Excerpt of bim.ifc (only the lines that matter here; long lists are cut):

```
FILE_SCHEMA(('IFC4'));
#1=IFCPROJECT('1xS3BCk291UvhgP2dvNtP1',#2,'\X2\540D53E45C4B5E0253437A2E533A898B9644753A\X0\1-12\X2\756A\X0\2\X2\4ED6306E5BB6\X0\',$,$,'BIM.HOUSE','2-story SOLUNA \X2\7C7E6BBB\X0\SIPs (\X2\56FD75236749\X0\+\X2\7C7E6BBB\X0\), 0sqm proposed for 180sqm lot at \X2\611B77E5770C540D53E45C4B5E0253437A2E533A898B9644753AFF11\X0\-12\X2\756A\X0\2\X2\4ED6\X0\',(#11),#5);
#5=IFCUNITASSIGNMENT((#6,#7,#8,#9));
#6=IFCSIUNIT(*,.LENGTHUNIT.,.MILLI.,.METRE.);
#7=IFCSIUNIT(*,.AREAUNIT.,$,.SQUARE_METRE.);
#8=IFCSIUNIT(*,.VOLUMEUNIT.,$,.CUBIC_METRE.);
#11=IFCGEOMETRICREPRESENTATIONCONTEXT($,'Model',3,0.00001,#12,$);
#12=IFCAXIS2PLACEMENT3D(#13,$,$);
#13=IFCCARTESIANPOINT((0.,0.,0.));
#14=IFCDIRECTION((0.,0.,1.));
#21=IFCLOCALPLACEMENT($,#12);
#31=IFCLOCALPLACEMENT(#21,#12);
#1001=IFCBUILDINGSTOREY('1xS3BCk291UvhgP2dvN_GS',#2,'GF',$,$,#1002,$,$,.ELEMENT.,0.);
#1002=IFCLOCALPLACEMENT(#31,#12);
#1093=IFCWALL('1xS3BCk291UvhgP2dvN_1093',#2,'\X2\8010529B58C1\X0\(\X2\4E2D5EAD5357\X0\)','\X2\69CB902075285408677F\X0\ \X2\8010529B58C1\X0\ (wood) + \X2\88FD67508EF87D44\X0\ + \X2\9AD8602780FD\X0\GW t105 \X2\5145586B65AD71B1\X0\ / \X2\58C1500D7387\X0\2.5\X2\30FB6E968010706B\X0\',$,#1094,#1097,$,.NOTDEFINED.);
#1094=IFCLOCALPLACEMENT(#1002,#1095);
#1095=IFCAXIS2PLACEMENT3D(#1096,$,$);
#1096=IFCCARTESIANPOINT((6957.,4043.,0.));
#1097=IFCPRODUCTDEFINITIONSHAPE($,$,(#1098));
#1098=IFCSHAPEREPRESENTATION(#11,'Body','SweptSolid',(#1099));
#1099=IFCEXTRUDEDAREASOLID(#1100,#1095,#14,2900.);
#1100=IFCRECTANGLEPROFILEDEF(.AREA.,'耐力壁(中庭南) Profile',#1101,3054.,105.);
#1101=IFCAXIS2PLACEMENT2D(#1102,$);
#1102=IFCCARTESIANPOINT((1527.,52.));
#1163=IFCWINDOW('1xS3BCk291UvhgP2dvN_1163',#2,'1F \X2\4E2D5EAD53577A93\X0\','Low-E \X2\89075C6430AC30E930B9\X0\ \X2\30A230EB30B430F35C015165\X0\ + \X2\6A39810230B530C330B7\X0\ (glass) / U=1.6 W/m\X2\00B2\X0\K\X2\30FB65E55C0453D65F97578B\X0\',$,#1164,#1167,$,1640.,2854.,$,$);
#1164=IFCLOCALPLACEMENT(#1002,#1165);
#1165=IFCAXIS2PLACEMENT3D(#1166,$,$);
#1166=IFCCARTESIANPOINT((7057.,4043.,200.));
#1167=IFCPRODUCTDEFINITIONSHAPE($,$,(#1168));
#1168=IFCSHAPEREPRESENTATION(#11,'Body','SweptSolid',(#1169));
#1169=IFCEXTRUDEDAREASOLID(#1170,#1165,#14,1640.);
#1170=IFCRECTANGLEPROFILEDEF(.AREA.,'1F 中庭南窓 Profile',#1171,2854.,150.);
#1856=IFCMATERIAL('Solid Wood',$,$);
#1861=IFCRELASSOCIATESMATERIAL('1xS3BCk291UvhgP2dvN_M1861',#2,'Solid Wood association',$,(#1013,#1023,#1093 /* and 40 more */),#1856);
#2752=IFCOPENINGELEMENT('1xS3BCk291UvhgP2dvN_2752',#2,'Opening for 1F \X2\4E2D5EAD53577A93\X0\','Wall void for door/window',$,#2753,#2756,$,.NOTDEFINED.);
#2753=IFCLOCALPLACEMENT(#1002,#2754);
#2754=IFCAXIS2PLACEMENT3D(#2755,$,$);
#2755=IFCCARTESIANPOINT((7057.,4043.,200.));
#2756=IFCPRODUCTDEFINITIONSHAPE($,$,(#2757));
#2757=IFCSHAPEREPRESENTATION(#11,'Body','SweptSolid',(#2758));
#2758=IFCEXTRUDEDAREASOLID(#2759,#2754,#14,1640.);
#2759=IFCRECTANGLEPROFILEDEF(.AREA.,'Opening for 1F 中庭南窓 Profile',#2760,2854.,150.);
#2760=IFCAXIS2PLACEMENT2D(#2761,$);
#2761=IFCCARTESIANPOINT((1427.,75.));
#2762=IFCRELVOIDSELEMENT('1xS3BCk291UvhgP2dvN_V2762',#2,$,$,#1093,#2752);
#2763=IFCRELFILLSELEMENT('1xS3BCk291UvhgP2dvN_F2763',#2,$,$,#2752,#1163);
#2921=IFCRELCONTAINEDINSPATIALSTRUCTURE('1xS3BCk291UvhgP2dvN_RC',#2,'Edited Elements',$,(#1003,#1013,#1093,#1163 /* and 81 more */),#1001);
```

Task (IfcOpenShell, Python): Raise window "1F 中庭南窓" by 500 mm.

```python
import numpy as np
import ifcopenshell
import ifcopenshell.api.geometry
import ifcopenshell.util.placement
import ifcopenshell.util.unit

model = ifcopenshell.open("bim.ifc")
unit_scale = ifcopenshell.util.unit.calculate_unit_scale(model)

window = model.by_id(1163)
opening = window.FillsVoids[0].RelatingOpeningElement
dz = 0.5 / unit_scale

shift = np.array([0.0, 0.0, dz])
# The window is not placed relative to its opening, so move both.
for product in (opening, window):
    matrix = ifcopenshell.util.placement.get_local_placement(product.ObjectPlacement)
    matrix[:3, 3] += shift
    ifcopenshell.api.geometry.edit_object_placement(model, product=product, matrix=matrix, is_si=False)

print(f"moved by {dz * unit_scale:+.3f} m")

model.write("bim_rev.ifc")
```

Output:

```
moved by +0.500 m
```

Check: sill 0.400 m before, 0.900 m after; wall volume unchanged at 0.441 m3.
